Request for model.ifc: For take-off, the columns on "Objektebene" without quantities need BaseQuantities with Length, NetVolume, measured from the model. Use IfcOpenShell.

First a look at what the model holds.

```python
import ifcopenshell
import ifcopenshell.util.element
import ifcopenshell.util.unit

model = ifcopenshell.open("model.ifc")
print(model.schema)
for unit_type in ("LENGTHUNIT", "AREAUNIT", "VOLUMEUNIT"):
    print(unit_type, ifcopenshell.util.unit.calculate_unit_scale(model, unit_type))
storey = next(s for s in model.by_type("IfcBuildingStorey") if s.Name == "Objektebene")
columns = [e for e in ifcopenshell.util.element.get_decomposition(storey) if e.is_a("IfcColumn")]
for e in sorted(columns, key=lambda e: e.id()):
    print(e.id(), e.is_a(), e.Name, list(ifcopenshell.util.element.get_psets(e, qtos_only=True)), sep=" | ")
```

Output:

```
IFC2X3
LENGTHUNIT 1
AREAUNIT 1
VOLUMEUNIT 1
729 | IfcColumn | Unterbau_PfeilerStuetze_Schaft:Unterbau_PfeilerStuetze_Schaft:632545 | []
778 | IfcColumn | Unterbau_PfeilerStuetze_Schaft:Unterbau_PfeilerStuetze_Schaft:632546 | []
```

```python
import ifcopenshell
import ifcopenshell.api.pset
import ifcopenshell.geom
import ifcopenshell.util.element
import ifcopenshell.util.shape
import ifcopenshell.util.unit

model = ifcopenshell.open("model.ifc")
unit_scale = ifcopenshell.util.unit.calculate_unit_scale(model)
volume_scale = ifcopenshell.util.unit.calculate_unit_scale(model, "VOLUMEUNIT")
settings = ifcopenshell.geom.settings()

storey = next(s for s in model.by_type("IfcBuildingStorey") if s.Name == "Objektebene")
columns = [e for e in ifcopenshell.util.element.get_decomposition(storey) if e.is_a("IfcColumn")]

for e in sorted(columns, key=lambda e: e.id()):
    if ifcopenshell.util.element.get_psets(e, qtos_only=True, should_inherit=False):
        continue
    # Geometry comes back in metres, in the element's own axes.
    shape = ifcopenshell.geom.create_shape(settings, e)
    values = {
        "Length": ifcopenshell.util.shape.get_z(shape.geometry) / unit_scale,
        "NetVolume": ifcopenshell.util.shape.get_volume(shape.geometry) / volume_scale,
    }
    qto = ifcopenshell.api.pset.add_qto(model, product=e, name="BaseQuantities")
    ifcopenshell.api.pset.edit_qto(model, qto=qto, properties=values)
    print(e.id(), {k: round(v, 3) for k, v in values.items()})

model.write("model_rev.ifc")
```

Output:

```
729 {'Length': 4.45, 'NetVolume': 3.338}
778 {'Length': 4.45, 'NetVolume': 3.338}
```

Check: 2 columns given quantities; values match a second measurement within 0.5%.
